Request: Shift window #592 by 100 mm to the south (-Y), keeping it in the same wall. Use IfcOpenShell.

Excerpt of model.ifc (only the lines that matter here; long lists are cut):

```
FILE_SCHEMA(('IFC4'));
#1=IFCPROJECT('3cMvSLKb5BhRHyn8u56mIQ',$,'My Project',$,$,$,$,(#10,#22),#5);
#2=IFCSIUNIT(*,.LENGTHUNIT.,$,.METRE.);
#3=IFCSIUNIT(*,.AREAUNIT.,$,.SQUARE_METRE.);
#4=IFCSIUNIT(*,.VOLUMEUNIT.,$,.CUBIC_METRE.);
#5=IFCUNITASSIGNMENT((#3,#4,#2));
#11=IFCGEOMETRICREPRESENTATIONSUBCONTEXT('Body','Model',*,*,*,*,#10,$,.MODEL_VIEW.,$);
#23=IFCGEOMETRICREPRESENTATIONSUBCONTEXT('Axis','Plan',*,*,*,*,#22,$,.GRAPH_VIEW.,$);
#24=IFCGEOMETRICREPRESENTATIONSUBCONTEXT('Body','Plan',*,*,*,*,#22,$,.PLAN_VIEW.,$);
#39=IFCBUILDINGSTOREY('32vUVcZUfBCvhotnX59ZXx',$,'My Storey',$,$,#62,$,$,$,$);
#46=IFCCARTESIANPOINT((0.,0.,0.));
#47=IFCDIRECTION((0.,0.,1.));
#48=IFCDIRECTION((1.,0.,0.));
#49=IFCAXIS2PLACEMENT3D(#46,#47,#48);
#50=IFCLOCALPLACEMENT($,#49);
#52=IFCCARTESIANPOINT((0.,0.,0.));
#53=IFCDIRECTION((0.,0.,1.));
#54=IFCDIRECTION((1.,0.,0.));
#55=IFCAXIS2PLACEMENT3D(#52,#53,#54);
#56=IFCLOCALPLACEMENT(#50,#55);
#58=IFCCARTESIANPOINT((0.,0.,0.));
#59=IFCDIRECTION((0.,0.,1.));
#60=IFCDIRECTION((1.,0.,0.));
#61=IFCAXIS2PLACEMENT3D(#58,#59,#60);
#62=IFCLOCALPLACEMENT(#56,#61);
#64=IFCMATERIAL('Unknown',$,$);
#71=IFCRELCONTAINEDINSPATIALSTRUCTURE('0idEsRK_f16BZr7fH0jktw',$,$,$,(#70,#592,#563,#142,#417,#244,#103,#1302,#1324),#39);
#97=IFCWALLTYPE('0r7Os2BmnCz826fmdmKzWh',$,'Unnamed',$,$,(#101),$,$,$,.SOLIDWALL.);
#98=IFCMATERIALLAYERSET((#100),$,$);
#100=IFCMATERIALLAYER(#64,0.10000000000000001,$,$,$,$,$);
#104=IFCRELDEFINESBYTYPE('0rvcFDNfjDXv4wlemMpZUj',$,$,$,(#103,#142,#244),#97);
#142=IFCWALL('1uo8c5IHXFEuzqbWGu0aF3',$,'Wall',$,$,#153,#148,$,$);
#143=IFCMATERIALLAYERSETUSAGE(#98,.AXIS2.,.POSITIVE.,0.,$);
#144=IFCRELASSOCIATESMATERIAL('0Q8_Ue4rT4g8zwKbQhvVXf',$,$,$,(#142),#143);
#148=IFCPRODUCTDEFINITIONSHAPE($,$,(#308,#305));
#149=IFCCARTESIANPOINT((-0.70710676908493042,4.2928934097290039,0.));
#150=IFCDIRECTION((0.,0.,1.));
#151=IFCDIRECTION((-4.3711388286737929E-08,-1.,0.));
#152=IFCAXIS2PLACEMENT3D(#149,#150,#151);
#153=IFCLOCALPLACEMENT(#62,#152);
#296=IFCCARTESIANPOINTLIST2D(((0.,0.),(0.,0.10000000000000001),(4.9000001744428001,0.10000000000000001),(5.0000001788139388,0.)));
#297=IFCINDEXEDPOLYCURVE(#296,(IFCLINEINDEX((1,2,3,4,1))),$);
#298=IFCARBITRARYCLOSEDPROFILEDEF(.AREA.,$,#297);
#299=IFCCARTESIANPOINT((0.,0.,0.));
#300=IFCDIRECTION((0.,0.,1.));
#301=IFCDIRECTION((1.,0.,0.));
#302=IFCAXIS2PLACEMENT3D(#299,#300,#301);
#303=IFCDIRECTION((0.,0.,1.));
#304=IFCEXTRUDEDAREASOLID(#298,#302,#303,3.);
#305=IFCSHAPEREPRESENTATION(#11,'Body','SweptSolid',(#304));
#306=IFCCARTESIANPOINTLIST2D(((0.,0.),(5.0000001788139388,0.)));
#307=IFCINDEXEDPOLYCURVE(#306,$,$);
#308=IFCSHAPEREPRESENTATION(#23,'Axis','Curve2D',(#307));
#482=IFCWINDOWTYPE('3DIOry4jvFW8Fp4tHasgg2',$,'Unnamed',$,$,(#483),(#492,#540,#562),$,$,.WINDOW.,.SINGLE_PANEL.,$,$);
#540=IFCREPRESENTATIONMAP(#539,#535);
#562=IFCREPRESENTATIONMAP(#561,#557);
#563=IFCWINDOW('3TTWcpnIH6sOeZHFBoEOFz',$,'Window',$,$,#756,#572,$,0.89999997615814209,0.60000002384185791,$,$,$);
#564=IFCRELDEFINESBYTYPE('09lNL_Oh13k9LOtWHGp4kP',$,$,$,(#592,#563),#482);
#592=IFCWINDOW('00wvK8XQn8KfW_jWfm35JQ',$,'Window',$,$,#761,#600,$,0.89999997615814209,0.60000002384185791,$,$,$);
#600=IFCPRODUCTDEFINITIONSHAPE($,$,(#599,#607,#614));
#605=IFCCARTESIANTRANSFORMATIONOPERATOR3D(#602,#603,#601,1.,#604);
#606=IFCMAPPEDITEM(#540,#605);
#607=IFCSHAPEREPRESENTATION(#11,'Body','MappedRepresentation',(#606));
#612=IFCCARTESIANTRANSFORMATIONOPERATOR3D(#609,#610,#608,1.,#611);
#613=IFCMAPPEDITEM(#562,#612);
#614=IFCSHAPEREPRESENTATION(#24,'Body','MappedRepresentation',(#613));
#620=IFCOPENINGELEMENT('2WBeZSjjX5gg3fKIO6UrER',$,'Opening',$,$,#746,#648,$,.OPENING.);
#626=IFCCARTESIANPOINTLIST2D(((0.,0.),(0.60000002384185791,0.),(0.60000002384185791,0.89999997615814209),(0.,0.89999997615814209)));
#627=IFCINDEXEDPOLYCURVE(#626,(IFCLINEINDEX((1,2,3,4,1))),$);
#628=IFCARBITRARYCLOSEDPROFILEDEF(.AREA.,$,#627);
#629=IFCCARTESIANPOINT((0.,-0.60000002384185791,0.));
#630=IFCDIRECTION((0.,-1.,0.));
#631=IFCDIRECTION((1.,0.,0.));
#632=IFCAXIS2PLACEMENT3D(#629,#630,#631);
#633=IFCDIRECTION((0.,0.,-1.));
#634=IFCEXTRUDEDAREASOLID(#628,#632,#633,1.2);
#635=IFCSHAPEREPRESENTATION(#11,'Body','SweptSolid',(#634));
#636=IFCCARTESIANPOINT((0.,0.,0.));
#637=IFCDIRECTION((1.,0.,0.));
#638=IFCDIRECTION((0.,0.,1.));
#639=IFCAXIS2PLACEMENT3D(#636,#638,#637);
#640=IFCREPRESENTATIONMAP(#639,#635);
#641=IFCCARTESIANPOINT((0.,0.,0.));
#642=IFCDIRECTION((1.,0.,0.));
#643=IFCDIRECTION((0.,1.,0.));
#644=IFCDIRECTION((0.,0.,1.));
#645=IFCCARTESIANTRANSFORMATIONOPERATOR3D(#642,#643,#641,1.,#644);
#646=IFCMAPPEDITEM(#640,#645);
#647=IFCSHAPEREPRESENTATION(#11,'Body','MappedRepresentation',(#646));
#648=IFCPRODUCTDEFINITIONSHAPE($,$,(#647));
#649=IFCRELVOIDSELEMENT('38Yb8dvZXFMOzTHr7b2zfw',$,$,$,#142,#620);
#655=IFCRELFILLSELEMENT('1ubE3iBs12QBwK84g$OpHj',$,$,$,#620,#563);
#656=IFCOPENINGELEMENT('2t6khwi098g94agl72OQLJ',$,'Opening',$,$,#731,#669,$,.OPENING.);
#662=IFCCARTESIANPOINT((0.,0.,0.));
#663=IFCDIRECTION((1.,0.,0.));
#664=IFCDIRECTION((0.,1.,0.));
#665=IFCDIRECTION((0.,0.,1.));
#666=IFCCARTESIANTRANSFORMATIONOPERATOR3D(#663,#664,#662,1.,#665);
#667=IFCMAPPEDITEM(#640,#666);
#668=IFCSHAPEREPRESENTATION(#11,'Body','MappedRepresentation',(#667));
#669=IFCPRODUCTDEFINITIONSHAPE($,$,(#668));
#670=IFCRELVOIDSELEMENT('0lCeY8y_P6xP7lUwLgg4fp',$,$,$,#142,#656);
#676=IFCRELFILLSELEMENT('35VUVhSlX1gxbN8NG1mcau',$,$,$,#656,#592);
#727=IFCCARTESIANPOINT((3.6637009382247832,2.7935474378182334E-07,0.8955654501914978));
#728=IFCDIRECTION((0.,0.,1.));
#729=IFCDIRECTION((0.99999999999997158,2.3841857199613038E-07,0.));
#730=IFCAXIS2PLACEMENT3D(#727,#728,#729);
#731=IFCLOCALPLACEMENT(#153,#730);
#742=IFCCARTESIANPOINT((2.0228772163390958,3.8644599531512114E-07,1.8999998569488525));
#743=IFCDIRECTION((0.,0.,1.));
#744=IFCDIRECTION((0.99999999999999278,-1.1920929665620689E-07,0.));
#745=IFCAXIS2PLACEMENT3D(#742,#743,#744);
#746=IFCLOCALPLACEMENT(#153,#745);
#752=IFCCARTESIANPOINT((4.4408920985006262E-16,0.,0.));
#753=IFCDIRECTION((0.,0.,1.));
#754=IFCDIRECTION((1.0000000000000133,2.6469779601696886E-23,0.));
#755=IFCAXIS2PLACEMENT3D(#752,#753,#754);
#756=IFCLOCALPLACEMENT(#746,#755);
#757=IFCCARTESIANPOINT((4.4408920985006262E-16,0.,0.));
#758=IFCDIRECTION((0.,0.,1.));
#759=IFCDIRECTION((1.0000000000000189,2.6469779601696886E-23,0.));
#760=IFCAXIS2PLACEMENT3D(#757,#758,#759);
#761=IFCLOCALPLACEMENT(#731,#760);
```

```python
import ifcopenshell
import ifcopenshell.api.geometry
import ifcopenshell.util.placement

model = ifcopenshell.open("model.ifc")

window = model.by_id(592)
opening = window.FillsVoids[0].RelatingOpeningElement
wall = opening.VoidsElements[0].RelatingBuildingElement

wall_matrix = ifcopenshell.util.placement.get_local_placement(wall.ObjectPlacement)
shift = wall_matrix[:3, 0] * 0.1
before = ifcopenshell.util.placement.get_local_placement(window.ObjectPlacement)[:3, 3].copy()

# The window is placed relative to its opening, so it follows when the opening moves.
matrix = ifcopenshell.util.placement.get_local_placement(opening.ObjectPlacement)
matrix[:3, 3] += shift
ifcopenshell.api.geometry.edit_object_placement(
    model, product=opening, matrix=matrix, is_si=False, should_transform_children=True
)

after = ifcopenshell.util.placement.get_local_placement(window.ObjectPlacement)[:3, 3]
print("window moved by", (after - before).round(3) + 0.0)

model.write("model_rev.ifc")
```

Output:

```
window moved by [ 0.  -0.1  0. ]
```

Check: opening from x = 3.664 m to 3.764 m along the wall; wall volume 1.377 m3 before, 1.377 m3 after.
